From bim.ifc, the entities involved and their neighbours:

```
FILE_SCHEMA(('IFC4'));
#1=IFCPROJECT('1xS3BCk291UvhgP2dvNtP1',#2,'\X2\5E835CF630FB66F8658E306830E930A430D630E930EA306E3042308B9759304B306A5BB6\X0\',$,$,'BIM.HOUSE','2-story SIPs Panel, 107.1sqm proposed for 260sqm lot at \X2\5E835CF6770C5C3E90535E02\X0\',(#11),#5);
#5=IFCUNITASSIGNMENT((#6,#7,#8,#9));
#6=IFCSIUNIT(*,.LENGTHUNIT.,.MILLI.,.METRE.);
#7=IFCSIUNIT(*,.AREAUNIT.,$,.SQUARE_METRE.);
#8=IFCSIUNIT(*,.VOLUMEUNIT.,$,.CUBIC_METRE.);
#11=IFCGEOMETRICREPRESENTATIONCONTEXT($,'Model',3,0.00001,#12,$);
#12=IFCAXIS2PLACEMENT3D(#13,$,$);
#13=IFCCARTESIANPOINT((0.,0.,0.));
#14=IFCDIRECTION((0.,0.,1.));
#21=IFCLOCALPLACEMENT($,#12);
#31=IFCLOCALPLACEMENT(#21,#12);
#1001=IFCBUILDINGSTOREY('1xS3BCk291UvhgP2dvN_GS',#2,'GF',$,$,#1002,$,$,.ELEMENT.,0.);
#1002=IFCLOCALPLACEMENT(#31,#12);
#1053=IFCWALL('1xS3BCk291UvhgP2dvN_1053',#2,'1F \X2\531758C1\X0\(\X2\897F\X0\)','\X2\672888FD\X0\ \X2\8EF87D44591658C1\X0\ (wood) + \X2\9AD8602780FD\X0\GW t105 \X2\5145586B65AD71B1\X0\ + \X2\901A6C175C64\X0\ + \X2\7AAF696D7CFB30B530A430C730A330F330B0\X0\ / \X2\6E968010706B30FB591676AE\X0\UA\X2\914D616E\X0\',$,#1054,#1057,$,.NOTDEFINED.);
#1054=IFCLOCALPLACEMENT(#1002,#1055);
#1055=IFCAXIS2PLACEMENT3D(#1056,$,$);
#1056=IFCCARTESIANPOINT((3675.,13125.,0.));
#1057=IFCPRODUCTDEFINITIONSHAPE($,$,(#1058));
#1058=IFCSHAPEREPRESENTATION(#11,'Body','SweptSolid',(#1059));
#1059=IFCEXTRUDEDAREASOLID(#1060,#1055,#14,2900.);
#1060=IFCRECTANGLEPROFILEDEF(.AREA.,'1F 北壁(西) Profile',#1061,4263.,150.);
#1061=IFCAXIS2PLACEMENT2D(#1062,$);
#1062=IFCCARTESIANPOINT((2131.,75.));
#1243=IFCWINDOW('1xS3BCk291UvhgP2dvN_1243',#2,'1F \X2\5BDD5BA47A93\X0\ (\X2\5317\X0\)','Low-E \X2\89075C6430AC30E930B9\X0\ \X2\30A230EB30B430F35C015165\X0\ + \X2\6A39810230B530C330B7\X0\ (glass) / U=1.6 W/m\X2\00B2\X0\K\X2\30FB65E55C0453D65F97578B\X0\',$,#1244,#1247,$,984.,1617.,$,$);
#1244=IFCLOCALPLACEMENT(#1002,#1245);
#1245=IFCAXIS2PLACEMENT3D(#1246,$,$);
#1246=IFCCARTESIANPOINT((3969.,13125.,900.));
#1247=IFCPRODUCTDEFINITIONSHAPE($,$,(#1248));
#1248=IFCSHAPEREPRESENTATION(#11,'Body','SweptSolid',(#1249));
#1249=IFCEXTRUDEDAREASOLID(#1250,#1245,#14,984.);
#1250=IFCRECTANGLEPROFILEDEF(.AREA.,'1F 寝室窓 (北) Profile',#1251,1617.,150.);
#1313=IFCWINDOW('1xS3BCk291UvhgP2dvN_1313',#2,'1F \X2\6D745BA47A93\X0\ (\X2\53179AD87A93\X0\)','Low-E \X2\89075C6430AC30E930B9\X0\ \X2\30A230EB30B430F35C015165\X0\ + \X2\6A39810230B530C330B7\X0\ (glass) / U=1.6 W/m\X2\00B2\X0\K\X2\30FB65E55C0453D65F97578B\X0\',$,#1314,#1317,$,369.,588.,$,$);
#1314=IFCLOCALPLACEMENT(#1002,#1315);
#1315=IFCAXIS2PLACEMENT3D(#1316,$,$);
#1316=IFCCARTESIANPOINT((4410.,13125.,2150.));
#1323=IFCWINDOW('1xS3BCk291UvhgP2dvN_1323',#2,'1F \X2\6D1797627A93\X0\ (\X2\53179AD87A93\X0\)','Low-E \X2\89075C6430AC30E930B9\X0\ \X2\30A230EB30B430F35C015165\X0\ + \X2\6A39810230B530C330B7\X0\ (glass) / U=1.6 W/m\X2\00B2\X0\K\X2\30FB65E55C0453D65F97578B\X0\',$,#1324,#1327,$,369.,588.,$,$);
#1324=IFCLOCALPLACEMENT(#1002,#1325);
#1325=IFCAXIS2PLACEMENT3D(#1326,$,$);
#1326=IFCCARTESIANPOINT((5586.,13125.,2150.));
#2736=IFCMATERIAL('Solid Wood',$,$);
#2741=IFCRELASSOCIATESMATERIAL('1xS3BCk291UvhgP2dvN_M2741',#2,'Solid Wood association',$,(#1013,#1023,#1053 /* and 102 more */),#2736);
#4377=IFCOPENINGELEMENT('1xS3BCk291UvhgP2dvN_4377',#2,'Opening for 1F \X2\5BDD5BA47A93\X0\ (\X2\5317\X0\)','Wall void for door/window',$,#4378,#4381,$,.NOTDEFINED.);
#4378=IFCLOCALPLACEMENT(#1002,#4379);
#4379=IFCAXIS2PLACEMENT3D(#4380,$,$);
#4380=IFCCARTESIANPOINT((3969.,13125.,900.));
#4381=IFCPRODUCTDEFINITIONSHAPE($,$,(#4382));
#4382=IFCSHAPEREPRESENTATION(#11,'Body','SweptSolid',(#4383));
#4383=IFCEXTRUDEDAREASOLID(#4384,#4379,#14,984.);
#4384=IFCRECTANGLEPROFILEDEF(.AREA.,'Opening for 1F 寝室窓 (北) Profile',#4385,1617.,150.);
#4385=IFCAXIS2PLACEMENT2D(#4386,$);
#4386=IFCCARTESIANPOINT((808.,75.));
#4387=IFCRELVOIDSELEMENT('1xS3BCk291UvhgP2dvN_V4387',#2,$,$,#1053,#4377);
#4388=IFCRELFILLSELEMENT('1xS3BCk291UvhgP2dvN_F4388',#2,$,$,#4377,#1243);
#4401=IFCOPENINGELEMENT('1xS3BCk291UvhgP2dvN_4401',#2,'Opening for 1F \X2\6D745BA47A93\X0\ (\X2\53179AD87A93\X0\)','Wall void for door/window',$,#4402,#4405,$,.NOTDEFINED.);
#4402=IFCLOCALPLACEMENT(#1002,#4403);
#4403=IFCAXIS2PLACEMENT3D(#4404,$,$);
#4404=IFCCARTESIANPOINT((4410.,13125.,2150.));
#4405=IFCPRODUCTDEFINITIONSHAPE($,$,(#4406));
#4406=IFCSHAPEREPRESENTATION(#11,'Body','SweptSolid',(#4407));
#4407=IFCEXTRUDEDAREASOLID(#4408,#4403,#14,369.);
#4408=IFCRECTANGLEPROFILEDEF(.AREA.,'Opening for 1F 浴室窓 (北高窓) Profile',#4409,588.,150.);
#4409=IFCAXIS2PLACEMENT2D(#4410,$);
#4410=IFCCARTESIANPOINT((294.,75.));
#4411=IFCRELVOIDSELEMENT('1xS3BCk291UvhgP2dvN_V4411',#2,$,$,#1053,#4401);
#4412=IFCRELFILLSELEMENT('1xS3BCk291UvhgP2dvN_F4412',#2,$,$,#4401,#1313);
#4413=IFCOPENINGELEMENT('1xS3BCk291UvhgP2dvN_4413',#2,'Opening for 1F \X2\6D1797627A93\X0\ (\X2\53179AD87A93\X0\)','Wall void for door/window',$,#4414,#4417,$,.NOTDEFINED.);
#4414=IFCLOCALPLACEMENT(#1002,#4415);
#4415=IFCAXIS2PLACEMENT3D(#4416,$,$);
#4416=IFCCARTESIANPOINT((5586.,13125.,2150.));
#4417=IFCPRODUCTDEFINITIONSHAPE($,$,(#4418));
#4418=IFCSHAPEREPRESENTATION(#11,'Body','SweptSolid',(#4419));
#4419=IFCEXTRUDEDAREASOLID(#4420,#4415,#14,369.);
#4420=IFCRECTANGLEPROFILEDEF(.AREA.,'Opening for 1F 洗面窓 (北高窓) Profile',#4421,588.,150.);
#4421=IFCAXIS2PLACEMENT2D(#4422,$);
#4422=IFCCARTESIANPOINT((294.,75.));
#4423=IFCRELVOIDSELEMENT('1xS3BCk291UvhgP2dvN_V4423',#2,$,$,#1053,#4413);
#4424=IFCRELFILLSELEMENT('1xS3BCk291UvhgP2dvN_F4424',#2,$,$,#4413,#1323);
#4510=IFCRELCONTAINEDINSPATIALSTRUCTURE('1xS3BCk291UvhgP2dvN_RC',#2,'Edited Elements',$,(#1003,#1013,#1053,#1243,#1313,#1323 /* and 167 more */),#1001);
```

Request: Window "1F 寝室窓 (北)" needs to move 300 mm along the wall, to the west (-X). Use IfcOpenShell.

```python
import ifcopenshell
import ifcopenshell.api.geometry
import ifcopenshell.util.placement
import ifcopenshell.util.unit

model = ifcopenshell.open("bim.ifc")
unit_scale = ifcopenshell.util.unit.calculate_unit_scale(model)

window = model.by_guid("1xS3BCk291UvhgP2dvN_1243")
opening = window.FillsVoids[0].RelatingOpeningElement
wall = opening.VoidsElements[0].RelatingBuildingElement

wall_matrix = ifcopenshell.util.placement.get_local_placement(wall.ObjectPlacement)
shift = wall_matrix[:3, 0] * -0.3 / unit_scale
before = ifcopenshell.util.placement.get_local_placement(window.ObjectPlacement)[:3, 3].copy()

# The window is not placed relative to its opening, so move both.
for product in (opening, window):
    matrix = ifcopenshell.util.placement.get_local_placement(product.ObjectPlacement)
    matrix[:3, 3] += shift
    ifcopenshell.api.geometry.edit_object_placement(model, product=product, matrix=matrix, is_si=False)

after = ifcopenshell.util.placement.get_local_placement(window.ObjectPlacement)[:3, 3]
print("window moved by", (after - before).round(3) + 0.0)

model.write("bim_v2.ifc")
```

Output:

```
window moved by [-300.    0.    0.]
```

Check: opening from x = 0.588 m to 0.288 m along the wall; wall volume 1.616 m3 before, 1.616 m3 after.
